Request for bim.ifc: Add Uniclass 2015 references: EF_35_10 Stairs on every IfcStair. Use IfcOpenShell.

First a look at what the model holds.

```python
import ifcopenshell

model = ifcopenshell.open("bim.ifc")
print(model.schema)
print("classifications:", [c.Name for c in model.by_type("IfcClassification")])
for ifc_class in ("IfcDoor", "IfcRoof", "IfcStair", "IfcWall", "IfcWindow"):
    print(ifc_class, len(model.by_type(ifc_class)))
```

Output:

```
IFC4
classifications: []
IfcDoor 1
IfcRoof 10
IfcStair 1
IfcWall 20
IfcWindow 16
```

```python
import ifcopenshell
import ifcopenshell.api.classification

model = ifcopenshell.open("bim.ifc")

system = ifcopenshell.api.classification.add_classification(model, classification="Uniclass 2015")

codes = {
    "IfcStair": ("EF_35_10", "Stairs"),
}
for ifc_class, (code, name) in codes.items():
    products = model.by_type(ifc_class)
    ifcopenshell.api.classification.add_reference(
        model, products=products, classification=system, identification=code, name=name
    )
    print(code, len(products))

model.write("bim_rev.ifc")
```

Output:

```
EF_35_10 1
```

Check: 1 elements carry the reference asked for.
